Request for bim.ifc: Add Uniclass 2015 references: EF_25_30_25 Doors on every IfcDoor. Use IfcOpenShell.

First a look at what the model holds.

```python
import ifcopenshell

model = ifcopenshell.open("bim.ifc")
print(model.schema)
print("classifications:", [c.Name for c in model.by_type("IfcClassification")])
for ifc_class in ("IfcDoor", "IfcRoof", "IfcStair", "IfcWall", "IfcWindow"):
    print(ifc_class, len(model.by_type(ifc_class)))
```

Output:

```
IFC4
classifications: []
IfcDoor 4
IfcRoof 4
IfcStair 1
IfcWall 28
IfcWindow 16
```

```python
import ifcopenshell
import ifcopenshell.api.classification

model = ifcopenshell.open("bim.ifc")

system = ifcopenshell.api.classification.add_classification(model, classification="Uniclass 2015")

codes = {
    "IfcDoor": ("EF_25_30_25", "Doors"),
}
for ifc_class, (code, name) in codes.items():
    products = model.by_type(ifc_class)
    ifcopenshell.api.classification.add_reference(
        model, products=products, classification=system, identification=code, name=name
    )
    print(code, len(products))

model.write("bim-out.ifc")
```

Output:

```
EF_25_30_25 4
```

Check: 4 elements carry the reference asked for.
